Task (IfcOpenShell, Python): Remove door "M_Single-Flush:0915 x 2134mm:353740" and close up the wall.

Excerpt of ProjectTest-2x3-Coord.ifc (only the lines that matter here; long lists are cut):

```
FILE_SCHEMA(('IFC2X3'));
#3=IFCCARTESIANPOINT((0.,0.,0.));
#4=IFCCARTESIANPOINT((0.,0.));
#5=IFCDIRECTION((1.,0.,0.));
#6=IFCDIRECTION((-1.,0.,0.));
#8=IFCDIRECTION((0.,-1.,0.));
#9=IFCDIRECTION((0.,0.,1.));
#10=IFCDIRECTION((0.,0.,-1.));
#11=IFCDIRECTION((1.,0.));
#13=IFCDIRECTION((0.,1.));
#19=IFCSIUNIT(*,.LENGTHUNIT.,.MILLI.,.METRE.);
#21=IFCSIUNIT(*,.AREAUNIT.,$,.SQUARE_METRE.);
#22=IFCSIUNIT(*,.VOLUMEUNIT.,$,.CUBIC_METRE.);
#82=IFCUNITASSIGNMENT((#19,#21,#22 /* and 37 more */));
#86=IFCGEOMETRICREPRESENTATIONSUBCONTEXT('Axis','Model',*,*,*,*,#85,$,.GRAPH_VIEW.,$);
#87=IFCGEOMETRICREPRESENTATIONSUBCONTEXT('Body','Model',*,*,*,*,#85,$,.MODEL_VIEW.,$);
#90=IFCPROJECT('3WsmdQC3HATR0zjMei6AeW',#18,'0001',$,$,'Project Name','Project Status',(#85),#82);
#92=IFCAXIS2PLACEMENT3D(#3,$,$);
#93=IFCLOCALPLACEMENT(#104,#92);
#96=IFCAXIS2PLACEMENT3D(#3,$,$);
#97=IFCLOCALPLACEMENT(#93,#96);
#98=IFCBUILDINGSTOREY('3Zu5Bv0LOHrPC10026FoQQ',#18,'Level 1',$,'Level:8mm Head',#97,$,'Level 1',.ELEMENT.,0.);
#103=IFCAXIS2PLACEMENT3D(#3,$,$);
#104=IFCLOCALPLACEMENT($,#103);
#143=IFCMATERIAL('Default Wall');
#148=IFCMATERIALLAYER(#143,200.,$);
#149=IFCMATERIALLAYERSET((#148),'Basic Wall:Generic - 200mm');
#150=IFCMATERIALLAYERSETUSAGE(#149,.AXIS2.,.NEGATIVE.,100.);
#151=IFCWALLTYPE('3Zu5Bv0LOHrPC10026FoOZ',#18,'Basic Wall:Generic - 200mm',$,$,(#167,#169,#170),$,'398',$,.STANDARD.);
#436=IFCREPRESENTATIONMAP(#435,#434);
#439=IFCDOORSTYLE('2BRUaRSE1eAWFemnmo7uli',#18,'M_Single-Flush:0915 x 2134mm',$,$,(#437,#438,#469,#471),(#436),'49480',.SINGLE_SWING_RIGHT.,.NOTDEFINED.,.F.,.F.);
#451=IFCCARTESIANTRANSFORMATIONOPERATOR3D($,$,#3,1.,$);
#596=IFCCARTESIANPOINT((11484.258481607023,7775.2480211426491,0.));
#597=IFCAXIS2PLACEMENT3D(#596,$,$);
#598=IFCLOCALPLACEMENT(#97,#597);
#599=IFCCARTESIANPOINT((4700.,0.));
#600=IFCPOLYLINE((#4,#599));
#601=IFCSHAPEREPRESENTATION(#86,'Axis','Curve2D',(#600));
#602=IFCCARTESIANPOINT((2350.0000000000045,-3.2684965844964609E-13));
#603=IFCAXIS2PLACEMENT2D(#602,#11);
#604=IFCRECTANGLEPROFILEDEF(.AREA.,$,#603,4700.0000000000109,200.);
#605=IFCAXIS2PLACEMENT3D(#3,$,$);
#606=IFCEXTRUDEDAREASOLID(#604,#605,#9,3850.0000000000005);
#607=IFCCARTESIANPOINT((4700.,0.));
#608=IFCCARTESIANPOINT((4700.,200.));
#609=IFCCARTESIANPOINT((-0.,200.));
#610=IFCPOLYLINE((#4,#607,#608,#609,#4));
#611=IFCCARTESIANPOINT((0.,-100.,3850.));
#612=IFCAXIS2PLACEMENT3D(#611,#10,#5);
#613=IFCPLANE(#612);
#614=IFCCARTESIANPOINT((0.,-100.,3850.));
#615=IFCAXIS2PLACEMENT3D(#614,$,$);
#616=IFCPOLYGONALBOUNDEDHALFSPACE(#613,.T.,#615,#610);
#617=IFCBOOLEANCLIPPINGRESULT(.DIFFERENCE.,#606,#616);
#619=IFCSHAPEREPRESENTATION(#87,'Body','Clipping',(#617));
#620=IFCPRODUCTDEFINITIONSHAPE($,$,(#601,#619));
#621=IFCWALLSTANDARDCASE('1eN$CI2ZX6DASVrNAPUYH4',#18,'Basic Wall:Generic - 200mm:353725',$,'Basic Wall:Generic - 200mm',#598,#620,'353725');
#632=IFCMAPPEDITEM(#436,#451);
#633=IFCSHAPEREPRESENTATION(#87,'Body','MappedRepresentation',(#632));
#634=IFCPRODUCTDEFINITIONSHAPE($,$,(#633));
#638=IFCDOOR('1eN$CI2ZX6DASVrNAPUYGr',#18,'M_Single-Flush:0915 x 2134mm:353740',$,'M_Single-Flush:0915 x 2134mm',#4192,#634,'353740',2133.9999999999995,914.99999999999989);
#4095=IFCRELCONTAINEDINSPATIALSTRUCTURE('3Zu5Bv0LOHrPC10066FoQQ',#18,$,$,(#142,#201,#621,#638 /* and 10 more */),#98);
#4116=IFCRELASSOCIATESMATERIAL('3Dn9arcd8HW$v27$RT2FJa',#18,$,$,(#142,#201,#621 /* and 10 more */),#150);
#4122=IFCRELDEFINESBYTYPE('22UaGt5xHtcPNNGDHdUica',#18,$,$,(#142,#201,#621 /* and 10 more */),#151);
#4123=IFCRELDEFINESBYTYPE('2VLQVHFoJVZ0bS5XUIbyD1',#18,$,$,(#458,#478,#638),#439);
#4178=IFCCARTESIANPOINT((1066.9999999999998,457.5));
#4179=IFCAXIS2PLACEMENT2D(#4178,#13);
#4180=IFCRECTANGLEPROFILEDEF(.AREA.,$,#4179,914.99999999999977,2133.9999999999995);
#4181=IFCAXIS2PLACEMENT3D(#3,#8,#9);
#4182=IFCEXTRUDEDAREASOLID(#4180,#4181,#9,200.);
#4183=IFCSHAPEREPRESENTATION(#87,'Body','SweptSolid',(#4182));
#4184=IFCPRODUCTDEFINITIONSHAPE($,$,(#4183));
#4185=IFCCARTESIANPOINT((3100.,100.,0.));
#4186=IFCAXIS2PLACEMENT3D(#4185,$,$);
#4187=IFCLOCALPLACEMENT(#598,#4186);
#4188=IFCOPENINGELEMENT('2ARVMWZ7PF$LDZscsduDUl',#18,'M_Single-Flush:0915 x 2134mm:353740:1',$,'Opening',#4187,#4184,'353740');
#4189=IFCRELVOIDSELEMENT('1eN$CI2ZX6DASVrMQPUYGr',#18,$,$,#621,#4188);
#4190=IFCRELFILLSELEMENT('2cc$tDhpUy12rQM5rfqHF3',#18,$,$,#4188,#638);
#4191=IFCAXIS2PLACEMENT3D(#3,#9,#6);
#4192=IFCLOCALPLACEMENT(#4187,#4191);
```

```python
import ifcopenshell
import ifcopenshell.api.feature
import ifcopenshell.api.root
import ifcopenshell.geom
import ifcopenshell.util.shape

model = ifcopenshell.open("ProjectTest-2x3-Coord.ifc")
settings = ifcopenshell.geom.settings()


def volume(element):
    """Net volume in cubic metres, openings subtracted."""
    shape = ifcopenshell.geom.create_shape(settings, element)
    return ifcopenshell.util.shape.get_volume(shape.geometry)


door = model.by_guid("1eN$CI2ZX6DASVrNAPUYGr")
opening = door.FillsVoids[0].RelatingOpeningElement
wall = opening.VoidsElements[0].RelatingBuildingElement
before = volume(wall)

ifcopenshell.api.root.remove_product(model, product=door)
ifcopenshell.api.feature.remove_feature(model, feature=opening)

after = volume(wall)

print(f"wall volume {before:.3f} -> {after:.3f} m3")

model.write("ProjectTest-2x3-Coord_v2.ifc")
```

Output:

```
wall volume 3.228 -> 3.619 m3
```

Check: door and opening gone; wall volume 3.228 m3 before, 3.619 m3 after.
